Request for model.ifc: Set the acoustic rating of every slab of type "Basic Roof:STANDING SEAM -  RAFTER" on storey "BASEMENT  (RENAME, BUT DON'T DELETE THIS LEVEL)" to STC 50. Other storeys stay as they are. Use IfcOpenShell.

First a look at what the model holds.

```python
import ifcopenshell
import ifcopenshell.util.element

model = ifcopenshell.open("model.ifc")
print(model.schema)
storey = next(s for s in model.by_type("IfcBuildingStorey") if s.Name == "BASEMENT  (RENAME, BUT DON'T DELETE THIS LEVEL)")
slabs = [e for e in ifcopenshell.util.element.get_decomposition(storey) if e.is_a("IfcSlab")]
seen = {}
for e in slabs:
    element_type = ifcopenshell.util.element.get_type(e)
    key = (element_type.Name if element_type != e and element_type else None, ifcopenshell.util.element.get_pset(e, "Pset_SlabCommon", "AcousticRating"))
    seen[key] = seen.get(key, 0) + 1
for (name, value), count in sorted(seen.items(), key=str):
    print(count, "x", name, "|", value)
```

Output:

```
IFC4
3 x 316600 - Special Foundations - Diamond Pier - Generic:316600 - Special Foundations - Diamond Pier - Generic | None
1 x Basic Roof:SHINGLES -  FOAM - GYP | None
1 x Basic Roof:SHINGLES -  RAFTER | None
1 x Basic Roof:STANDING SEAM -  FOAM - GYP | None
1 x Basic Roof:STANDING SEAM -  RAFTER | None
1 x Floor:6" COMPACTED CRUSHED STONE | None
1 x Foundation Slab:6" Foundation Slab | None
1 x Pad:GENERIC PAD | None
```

```python
import ifcopenshell
import ifcopenshell.api.pset
import ifcopenshell.util.element

model = ifcopenshell.open("model.ifc")

storey = next(s for s in model.by_type("IfcBuildingStorey") if s.Name == "BASEMENT  (RENAME, BUT DON'T DELETE THIS LEVEL)")
slabs = [e for e in ifcopenshell.util.element.get_decomposition(storey) if e.is_a("IfcSlab")]

count = 0
for e in slabs:
    element_type = ifcopenshell.util.element.get_type(e)
    if element_type in (None, e) or element_type.Name != "Basic Roof:STANDING SEAM -  RAFTER":
        continue
    # add_pset returns the element's existing set when there is one.
    pset = ifcopenshell.api.pset.add_pset(model, product=e, name="Pset_SlabCommon")
    ifcopenshell.api.pset.edit_pset(model, pset=pset, properties={"AcousticRating": "STC 50"})
    count += 1

print(count, "slabs updated")

model.write("model-out.ifc")
```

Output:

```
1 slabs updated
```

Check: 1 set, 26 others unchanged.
